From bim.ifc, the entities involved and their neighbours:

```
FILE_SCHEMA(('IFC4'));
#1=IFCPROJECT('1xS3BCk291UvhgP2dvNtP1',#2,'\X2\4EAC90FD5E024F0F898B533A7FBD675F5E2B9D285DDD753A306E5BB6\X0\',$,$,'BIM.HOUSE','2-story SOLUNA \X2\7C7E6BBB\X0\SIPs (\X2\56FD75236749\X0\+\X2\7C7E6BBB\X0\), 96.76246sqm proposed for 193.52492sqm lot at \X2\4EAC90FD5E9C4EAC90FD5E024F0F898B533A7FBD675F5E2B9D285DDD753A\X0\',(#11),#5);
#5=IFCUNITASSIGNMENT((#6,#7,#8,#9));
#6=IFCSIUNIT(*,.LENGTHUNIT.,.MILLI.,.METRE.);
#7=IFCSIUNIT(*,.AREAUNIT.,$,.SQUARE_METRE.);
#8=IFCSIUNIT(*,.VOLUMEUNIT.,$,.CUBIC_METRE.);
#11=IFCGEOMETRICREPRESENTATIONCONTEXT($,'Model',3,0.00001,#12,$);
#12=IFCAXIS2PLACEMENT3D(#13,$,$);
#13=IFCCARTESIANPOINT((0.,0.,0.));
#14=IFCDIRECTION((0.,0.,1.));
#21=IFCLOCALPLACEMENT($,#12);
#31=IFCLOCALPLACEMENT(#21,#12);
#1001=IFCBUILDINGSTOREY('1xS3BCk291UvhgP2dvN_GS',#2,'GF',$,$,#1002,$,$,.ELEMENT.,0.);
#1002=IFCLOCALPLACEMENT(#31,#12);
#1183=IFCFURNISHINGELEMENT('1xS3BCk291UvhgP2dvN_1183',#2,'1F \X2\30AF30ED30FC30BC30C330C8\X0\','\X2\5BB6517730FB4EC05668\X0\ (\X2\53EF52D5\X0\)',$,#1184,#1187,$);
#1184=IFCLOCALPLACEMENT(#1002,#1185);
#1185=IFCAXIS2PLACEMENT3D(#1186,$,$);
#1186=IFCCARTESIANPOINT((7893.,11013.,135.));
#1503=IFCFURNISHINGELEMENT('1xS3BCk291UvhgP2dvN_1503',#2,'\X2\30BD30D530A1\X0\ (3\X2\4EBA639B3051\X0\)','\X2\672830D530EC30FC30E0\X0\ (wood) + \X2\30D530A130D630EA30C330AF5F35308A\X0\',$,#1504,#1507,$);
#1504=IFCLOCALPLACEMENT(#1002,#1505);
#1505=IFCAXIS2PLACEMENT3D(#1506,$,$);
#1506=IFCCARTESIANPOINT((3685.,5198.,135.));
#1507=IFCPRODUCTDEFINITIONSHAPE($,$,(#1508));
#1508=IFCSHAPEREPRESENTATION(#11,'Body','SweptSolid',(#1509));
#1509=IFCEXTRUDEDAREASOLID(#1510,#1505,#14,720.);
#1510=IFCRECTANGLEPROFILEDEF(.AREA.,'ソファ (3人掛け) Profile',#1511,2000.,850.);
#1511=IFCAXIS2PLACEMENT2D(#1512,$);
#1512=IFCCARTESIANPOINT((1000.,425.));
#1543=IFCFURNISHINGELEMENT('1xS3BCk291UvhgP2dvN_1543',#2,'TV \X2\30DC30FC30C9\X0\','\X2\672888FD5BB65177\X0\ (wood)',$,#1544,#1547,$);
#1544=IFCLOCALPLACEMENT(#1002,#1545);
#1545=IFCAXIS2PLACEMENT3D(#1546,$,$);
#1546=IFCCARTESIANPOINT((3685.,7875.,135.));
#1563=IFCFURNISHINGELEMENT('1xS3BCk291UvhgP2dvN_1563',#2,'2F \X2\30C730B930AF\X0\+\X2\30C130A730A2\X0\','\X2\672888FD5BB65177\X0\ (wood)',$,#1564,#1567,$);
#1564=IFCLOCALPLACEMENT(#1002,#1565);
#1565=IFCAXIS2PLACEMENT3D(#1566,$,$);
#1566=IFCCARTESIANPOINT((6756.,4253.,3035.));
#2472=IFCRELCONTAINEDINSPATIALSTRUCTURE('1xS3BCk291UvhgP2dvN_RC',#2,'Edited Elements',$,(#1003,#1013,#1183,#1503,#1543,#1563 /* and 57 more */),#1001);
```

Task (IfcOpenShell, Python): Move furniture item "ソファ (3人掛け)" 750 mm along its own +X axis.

```python
import ifcopenshell
import ifcopenshell.api.geometry
import ifcopenshell.util.placement
import ifcopenshell.util.unit

model = ifcopenshell.open("bim.ifc")
unit_scale = ifcopenshell.util.unit.calculate_unit_scale(model)

item = model.by_guid("1xS3BCk291UvhgP2dvN_1503")
matrix = ifcopenshell.util.placement.get_local_placement(item.ObjectPlacement)
matrix[:3, 3] += matrix[:3, 0] * 0.75 / unit_scale
ifcopenshell.api.geometry.edit_object_placement(model, product=item, matrix=matrix, is_si=False)

print(ifcopenshell.util.placement.get_local_placement(item.ObjectPlacement).round(3) + 0.0)

model.write("bim_rev.ifc")
```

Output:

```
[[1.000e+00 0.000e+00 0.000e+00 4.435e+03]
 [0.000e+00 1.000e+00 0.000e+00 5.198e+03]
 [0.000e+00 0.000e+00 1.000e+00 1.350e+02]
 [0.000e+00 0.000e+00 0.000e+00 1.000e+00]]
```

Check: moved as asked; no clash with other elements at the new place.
